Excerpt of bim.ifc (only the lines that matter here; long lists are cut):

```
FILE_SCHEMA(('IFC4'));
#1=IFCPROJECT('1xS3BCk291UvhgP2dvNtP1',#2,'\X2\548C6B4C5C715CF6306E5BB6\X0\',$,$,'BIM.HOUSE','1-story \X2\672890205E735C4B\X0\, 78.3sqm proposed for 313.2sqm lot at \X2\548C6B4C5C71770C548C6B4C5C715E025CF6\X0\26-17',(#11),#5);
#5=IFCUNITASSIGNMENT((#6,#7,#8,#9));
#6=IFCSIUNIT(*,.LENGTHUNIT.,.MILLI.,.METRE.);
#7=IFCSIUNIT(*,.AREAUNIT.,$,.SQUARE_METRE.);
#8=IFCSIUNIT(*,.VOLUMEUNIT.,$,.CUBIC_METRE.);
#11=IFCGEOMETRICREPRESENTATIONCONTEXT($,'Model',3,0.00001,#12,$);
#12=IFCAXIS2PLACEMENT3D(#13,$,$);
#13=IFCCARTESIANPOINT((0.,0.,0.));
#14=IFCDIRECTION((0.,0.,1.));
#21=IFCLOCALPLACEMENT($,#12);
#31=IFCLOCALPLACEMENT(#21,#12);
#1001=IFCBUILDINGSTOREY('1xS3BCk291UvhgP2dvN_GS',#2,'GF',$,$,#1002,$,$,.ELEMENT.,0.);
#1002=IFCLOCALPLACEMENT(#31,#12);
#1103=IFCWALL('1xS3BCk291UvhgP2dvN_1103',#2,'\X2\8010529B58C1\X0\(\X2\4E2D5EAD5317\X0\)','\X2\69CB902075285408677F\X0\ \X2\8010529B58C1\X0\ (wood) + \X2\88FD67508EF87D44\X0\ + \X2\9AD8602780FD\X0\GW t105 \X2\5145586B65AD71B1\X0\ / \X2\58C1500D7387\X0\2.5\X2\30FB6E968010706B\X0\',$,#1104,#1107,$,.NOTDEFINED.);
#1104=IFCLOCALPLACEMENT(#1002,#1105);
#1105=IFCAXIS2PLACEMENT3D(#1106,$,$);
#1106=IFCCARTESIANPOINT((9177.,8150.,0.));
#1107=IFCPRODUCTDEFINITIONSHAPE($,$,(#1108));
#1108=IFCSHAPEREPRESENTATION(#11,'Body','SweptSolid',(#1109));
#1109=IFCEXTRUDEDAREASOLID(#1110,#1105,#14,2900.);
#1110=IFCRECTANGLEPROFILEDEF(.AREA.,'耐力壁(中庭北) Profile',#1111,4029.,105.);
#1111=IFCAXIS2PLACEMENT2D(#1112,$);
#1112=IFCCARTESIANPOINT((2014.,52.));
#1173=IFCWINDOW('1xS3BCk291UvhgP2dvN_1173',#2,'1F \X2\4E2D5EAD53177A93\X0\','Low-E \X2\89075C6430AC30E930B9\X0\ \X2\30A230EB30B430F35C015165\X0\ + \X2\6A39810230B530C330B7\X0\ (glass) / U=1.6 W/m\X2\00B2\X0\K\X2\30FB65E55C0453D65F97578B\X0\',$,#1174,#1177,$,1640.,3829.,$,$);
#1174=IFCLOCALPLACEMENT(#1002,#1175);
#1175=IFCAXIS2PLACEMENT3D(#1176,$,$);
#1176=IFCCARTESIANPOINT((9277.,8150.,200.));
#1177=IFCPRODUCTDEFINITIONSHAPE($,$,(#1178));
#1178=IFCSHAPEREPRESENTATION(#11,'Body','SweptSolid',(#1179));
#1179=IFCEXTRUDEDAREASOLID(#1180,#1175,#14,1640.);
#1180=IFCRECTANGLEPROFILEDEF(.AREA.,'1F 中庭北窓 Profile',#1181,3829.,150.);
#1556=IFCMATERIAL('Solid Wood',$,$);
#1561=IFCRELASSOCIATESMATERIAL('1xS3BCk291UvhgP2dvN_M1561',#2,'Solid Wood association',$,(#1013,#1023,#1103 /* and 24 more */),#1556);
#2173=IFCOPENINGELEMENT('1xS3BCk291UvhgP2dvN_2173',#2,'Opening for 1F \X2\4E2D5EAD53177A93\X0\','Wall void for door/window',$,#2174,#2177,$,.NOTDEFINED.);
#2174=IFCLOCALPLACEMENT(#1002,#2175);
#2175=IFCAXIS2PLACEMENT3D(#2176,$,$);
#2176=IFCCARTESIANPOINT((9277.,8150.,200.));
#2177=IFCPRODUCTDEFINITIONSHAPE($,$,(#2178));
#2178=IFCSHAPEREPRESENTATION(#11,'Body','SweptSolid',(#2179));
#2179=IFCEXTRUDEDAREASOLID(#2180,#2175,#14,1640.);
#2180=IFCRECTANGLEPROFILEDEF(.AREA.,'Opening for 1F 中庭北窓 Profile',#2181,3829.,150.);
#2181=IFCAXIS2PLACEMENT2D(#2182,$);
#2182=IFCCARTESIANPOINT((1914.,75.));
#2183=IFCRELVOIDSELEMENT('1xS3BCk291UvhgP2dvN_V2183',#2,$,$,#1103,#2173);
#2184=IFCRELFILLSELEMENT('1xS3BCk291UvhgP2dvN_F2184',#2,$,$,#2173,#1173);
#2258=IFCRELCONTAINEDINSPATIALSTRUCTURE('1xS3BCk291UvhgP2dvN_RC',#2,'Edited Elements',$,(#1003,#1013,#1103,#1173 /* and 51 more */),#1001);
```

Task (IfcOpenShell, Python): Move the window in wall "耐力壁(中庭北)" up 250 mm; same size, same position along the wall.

```python
import numpy as np
import ifcopenshell
import ifcopenshell.api.geometry
import ifcopenshell.util.placement
import ifcopenshell.util.unit

model = ifcopenshell.open("bim.ifc")
unit_scale = ifcopenshell.util.unit.calculate_unit_scale(model)

window = model.by_id(1173)
opening = window.FillsVoids[0].RelatingOpeningElement
dz = 250.0

shift = np.array([0.0, 0.0, dz])
# The window is not placed relative to its opening, so move both.
for product in (opening, window):
    matrix = ifcopenshell.util.placement.get_local_placement(product.ObjectPlacement)
    matrix[:3, 3] += shift
    ifcopenshell.api.geometry.edit_object_placement(model, product=product, matrix=matrix, is_si=False)

print(f"moved by {dz * unit_scale:+.3f} m")

model.write("bim-out.ifc")
```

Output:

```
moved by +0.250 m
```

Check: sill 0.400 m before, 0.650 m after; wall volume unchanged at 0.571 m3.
